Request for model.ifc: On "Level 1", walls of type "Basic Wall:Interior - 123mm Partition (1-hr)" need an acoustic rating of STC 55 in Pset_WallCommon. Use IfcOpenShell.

First a look at what the model holds.

```python
import ifcopenshell
import ifcopenshell.util.element

model = ifcopenshell.open("model.ifc")
print(model.schema)
storey = next(s for s in model.by_type("IfcBuildingStorey") if s.Name == "Level 1")
walls = [e for e in ifcopenshell.util.element.get_decomposition(storey) if e.is_a("IfcWall")]
seen = {}
for e in walls:
    element_type = ifcopenshell.util.element.get_type(e)
    key = (element_type.Name if element_type != e and element_type else None, ifcopenshell.util.element.get_pset(e, "Pset_WallCommon", "AcousticRating"))
    seen[key] = seen.get(key, 0) + 1
for (name, value), count in sorted(seen.items(), key=str):
    print(count, "x", name, "|", value)
```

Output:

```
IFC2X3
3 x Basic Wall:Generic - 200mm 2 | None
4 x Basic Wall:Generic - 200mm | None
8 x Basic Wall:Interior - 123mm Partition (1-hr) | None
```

```python
import ifcopenshell
import ifcopenshell.api.pset
import ifcopenshell.util.element

model = ifcopenshell.open("model.ifc")

storey = next(s for s in model.by_type("IfcBuildingStorey") if s.Name == "Level 1")
walls = [e for e in ifcopenshell.util.element.get_decomposition(storey) if e.is_a("IfcWall")]

count = 0
for e in walls:
    element_type = ifcopenshell.util.element.get_type(e)
    if element_type in (None, e) or element_type.Name != "Basic Wall:Interior - 123mm Partition (1-hr)":
        continue
    # add_pset returns the element's existing set when there is one.
    pset = ifcopenshell.api.pset.add_pset(model, product=e, name="Pset_WallCommon")
    ifcopenshell.api.pset.edit_pset(model, pset=pset, properties={"AcousticRating": "STC 55"})
    count += 1

print(count, "walls updated")

model.write("model_edited.ifc")
```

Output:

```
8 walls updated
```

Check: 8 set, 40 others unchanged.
